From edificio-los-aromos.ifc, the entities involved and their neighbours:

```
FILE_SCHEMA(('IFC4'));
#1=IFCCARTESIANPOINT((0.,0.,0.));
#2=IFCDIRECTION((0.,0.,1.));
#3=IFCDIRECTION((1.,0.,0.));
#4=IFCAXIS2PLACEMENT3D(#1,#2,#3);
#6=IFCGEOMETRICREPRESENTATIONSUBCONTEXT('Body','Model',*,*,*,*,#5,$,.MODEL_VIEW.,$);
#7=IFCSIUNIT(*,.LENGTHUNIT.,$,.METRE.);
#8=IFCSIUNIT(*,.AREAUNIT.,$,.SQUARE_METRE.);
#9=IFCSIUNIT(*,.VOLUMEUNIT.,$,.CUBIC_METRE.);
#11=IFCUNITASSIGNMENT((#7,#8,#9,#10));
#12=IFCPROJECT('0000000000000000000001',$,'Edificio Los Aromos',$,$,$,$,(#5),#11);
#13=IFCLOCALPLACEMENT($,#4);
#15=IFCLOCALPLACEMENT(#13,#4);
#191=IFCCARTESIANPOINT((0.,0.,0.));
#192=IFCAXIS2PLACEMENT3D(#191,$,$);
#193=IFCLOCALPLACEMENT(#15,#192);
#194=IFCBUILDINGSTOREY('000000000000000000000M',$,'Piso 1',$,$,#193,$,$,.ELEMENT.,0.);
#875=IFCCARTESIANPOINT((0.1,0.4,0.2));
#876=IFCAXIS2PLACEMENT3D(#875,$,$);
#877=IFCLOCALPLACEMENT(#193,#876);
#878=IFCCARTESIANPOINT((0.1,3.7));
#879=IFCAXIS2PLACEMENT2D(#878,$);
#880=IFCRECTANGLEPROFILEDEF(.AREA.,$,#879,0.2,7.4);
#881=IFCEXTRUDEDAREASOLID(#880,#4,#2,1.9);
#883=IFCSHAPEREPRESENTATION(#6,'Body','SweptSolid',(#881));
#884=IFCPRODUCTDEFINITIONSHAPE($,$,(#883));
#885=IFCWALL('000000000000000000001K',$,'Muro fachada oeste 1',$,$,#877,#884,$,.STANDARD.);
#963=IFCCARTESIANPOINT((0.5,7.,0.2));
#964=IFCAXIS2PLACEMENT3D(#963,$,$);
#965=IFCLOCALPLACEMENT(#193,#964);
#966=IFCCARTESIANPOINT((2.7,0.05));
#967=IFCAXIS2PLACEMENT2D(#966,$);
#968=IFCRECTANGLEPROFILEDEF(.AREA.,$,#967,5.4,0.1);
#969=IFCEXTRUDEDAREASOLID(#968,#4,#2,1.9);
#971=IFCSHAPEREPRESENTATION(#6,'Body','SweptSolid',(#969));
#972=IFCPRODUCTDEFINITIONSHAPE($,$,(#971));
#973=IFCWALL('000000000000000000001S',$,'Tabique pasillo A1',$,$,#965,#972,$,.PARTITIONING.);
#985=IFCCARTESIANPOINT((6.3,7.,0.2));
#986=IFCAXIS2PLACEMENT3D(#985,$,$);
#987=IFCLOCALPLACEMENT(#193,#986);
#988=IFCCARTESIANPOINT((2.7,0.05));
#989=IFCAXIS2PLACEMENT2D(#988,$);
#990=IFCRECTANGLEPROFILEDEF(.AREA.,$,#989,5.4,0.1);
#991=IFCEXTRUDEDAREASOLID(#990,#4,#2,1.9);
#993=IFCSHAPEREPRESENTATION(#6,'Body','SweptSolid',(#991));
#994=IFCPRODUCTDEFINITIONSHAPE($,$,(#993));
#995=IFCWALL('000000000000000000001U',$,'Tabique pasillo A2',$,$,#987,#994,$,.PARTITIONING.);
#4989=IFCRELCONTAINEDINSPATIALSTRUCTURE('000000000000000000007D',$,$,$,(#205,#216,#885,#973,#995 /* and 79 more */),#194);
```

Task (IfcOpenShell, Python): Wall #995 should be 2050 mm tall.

```python
import ifcopenshell
import ifcopenshell.geom
import ifcopenshell.util.representation
import ifcopenshell.util.shape
import ifcopenshell.util.unit

model = ifcopenshell.open("edificio-los-aromos.ifc")
unit_scale = ifcopenshell.util.unit.calculate_unit_scale(model)
settings = ifcopenshell.geom.settings()


def volume(element):
    """Net volume in cubic metres, openings subtracted."""
    shape = ifcopenshell.geom.create_shape(settings, element)
    return ifcopenshell.util.shape.get_volume(shape.geometry)


wall = model.by_guid("000000000000000000001U")
before = volume(wall)

body = ifcopenshell.util.representation.get_representation(wall, "Model", "Body")
solid = body.Items[0]
old_height = solid.Depth
solid.Depth = 2.05 / unit_scale
after = volume(wall)

print(f"height {old_height:g} -> {solid.Depth:g}, volume {before:.3f} -> {after:.3f} m3")

model.write("edificio-los-aromos_v2.ifc")
```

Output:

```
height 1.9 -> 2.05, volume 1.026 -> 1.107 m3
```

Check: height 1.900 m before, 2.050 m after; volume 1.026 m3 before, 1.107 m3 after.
